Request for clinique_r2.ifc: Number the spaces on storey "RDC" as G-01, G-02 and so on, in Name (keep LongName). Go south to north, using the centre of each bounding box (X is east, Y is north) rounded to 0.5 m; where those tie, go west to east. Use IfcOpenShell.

First a look at what the model holds.

```python
import ifcopenshell
import ifcopenshell.util.element
import ifcopenshell.util.placement

model = ifcopenshell.open("clinique_r2.ifc")
print(model.schema)
storey = next(s for s in model.by_type("IfcBuildingStorey") if s.Name == "RDC")
spaces = [e for e in ifcopenshell.util.element.get_decomposition(storey) if e.is_a("IfcSpace")]
for e in sorted(spaces, key=lambda e: e.id()):
    origin = ifcopenshell.util.placement.get_local_placement(e.ObjectPlacement)[:3, 3]
    print(e.id(), e.Name, e.LongName, origin.round(2) + 0.0, sep=" | ")
```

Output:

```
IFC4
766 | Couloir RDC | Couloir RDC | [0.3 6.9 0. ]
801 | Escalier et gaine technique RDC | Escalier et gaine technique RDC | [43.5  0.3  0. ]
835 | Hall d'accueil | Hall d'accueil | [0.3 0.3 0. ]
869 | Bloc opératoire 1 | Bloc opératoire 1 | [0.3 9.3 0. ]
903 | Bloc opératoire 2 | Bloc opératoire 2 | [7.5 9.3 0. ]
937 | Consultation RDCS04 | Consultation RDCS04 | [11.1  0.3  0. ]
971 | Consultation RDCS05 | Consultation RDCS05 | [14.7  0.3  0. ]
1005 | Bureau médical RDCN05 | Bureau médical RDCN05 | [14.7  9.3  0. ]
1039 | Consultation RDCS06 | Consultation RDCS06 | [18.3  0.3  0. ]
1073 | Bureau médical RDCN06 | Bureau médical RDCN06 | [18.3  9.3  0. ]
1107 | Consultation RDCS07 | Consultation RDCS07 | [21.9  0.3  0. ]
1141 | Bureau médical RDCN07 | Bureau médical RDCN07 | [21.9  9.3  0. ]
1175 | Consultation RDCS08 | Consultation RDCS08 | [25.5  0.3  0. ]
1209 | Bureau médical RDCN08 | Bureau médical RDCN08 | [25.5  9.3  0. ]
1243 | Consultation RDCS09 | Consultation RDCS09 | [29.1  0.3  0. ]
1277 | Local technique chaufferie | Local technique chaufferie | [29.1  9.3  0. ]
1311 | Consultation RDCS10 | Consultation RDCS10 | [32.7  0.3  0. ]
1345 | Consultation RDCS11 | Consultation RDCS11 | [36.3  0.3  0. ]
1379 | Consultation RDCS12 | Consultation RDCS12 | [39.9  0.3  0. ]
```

```python
import ifcopenshell
import ifcopenshell.geom
import ifcopenshell.util.element
import ifcopenshell.util.shape

model = ifcopenshell.open("clinique_r2.ifc")
settings = ifcopenshell.geom.settings()
settings.set("use-world-coords", True)


def centre(element):
    shape = ifcopenshell.geom.create_shape(settings, element)
    return ifcopenshell.util.shape.get_bbox_centroid(shape.geometry)


storey = next(s for s in model.by_type("IfcBuildingStorey") if s.Name == "RDC")
spaces = [e for e in ifcopenshell.util.element.get_decomposition(storey) if e.is_a("IfcSpace")]

# Insertion points can sit at a corner or the storey origin, so sort by the geometry (in metres).
centres = {e: centre(e) for e in spaces}
spaces.sort(key=lambda e: (round(centres[e][1] / 0.5), centres[e][0]))

for i, e in enumerate(spaces, start=1):
    number = f"G-{i:02d}"
    e.Name = number
    print(e.id(), number)

model.write("clinique_r2_updated.ifc")
```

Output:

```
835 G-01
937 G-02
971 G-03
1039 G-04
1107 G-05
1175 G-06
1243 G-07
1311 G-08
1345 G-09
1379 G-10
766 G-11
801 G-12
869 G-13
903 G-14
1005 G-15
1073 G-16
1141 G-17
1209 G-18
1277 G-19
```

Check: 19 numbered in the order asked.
